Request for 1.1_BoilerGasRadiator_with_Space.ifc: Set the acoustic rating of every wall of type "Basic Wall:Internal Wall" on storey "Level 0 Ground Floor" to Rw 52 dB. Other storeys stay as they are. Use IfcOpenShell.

First a look at what the model holds.

```python
import ifcopenshell
import ifcopenshell.util.element

model = ifcopenshell.open("1.1_BoilerGasRadiator_with_Space.ifc")
print(model.schema)
storey = next(s for s in model.by_type("IfcBuildingStorey") if s.Name == "Level 0 Ground Floor")
walls = [e for e in ifcopenshell.util.element.get_decomposition(storey) if e.is_a("IfcWall")]
seen = {}
for e in walls:
    element_type = ifcopenshell.util.element.get_type(e)
    key = (element_type.Name if element_type != e and element_type else None, ifcopenshell.util.element.get_pset(e, "Pset_WallCommon", "AcousticRating"))
    seen[key] = seen.get(key, 0) + 1
for (name, value), count in sorted(seen.items(), key=str):
    print(count, "x", name, "|", value)
```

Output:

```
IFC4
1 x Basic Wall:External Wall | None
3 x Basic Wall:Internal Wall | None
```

```python
import ifcopenshell
import ifcopenshell.api.pset
import ifcopenshell.util.element

model = ifcopenshell.open("1.1_BoilerGasRadiator_with_Space.ifc")

storey = next(s for s in model.by_type("IfcBuildingStorey") if s.Name == "Level 0 Ground Floor")
walls = [e for e in ifcopenshell.util.element.get_decomposition(storey) if e.is_a("IfcWall")]

count = 0
for e in walls:
    element_type = ifcopenshell.util.element.get_type(e)
    if element_type in (None, e) or element_type.Name != "Basic Wall:Internal Wall":
        continue
    # add_pset returns the element's existing set when there is one.
    pset = ifcopenshell.api.pset.add_pset(model, product=e, name="Pset_WallCommon")
    ifcopenshell.api.pset.edit_pset(model, pset=pset, properties={"AcousticRating": "Rw 52 dB"})
    count += 1

print(count, "walls updated")

model.write("1.1_BoilerGasRadiator_with_Space_edited.ifc")
```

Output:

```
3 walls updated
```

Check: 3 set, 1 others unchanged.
